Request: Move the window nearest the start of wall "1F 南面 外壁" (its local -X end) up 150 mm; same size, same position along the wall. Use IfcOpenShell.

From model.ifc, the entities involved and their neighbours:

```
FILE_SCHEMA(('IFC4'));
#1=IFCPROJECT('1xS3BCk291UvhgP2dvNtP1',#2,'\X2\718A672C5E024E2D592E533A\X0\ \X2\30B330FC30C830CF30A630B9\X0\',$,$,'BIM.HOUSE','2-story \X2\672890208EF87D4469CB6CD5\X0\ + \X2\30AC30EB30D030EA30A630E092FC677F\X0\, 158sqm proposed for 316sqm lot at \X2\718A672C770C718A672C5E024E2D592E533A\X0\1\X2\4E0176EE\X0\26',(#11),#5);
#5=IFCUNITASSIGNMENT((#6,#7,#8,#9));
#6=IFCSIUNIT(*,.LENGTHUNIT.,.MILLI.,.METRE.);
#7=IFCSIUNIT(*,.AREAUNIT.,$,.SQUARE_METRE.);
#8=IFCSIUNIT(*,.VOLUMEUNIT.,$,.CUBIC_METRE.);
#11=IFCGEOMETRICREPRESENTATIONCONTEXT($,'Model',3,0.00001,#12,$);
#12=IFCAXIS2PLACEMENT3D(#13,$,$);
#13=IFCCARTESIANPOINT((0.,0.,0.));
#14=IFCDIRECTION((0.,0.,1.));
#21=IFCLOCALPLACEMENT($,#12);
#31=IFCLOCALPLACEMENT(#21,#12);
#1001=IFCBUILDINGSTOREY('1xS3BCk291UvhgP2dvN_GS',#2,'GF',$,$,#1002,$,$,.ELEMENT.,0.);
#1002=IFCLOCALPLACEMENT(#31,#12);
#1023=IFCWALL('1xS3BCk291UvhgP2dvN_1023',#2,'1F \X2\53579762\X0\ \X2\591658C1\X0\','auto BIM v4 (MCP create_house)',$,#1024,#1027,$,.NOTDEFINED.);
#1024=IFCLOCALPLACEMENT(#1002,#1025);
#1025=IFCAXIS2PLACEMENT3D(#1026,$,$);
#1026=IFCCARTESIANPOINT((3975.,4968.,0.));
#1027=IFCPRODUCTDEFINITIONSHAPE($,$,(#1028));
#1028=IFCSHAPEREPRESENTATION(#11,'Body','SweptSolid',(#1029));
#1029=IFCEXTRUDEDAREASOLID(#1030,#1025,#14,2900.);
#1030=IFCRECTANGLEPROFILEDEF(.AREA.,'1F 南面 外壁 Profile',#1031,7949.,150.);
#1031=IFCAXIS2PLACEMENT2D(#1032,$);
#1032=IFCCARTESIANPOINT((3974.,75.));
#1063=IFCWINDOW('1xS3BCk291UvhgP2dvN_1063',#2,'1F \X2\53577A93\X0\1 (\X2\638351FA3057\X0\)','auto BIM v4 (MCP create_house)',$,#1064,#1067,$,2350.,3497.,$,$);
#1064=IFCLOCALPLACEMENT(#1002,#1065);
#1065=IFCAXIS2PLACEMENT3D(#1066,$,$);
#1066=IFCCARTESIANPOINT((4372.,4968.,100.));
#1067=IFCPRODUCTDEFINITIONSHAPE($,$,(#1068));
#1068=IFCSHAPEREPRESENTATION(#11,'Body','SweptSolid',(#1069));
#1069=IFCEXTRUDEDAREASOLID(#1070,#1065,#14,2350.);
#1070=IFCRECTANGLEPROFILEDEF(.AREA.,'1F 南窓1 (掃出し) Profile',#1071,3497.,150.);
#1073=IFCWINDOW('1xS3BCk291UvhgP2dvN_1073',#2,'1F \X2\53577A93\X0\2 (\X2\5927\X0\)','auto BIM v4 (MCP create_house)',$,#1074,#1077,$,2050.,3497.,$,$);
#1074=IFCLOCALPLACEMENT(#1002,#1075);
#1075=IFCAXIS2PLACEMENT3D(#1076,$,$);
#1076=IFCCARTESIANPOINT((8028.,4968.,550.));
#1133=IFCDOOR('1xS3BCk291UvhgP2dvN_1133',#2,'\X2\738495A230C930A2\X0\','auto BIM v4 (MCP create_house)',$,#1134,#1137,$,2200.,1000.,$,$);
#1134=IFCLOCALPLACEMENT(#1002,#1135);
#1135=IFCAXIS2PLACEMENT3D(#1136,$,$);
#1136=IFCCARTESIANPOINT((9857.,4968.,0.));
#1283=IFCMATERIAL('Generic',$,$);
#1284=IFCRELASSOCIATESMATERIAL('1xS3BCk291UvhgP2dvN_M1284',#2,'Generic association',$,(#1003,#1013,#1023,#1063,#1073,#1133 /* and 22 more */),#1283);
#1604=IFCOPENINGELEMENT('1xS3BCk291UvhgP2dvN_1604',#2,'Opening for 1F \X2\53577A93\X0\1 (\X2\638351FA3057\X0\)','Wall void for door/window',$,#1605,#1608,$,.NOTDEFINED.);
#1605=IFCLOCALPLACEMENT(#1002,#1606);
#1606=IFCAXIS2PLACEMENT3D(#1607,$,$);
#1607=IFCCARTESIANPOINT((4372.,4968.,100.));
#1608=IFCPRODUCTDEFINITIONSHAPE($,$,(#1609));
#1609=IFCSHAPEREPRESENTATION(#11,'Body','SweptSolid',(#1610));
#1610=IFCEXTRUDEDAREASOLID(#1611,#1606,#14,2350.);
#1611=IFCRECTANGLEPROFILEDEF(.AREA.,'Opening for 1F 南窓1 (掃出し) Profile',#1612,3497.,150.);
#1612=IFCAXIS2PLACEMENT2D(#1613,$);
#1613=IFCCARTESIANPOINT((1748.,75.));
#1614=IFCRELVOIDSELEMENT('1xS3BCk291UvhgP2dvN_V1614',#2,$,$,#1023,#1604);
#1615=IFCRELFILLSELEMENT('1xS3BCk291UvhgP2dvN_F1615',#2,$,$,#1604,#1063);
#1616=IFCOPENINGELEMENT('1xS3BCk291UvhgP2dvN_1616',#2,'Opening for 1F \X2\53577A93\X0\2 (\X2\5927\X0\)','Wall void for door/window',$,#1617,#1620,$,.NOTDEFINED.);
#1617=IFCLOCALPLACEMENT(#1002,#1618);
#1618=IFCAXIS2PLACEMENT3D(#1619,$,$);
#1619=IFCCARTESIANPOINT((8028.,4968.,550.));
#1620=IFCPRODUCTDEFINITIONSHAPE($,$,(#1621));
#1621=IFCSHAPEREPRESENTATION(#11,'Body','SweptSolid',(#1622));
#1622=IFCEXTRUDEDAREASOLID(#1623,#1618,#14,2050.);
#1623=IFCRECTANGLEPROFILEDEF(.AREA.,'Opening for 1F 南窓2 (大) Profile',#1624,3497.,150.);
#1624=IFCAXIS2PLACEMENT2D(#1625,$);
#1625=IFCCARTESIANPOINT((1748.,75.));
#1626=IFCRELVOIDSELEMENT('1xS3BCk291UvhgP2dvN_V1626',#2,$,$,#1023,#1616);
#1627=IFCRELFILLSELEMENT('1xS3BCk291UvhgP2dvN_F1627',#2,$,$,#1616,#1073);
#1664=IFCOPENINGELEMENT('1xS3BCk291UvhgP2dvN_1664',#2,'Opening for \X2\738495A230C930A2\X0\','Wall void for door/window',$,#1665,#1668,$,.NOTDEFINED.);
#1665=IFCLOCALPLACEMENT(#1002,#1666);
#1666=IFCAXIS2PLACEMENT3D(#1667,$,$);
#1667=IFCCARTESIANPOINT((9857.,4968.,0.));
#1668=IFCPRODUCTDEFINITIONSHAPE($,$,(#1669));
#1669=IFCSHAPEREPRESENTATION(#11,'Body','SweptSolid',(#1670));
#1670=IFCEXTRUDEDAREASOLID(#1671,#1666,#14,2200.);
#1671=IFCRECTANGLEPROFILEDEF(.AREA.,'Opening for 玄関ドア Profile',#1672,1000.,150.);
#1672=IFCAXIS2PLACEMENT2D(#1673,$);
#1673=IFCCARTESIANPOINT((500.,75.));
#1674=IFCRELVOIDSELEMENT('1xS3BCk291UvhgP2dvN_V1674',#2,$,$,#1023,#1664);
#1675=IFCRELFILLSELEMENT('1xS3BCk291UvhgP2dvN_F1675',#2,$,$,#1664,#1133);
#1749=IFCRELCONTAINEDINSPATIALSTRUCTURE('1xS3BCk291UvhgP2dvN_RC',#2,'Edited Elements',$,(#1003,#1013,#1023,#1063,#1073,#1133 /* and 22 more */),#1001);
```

```python
import numpy as np
import ifcopenshell
import ifcopenshell.api.geometry
import ifcopenshell.util.placement
import ifcopenshell.util.unit

model = ifcopenshell.open("model.ifc")
unit_scale = ifcopenshell.util.unit.calculate_unit_scale(model)

window = model.by_id(1063)
opening = window.FillsVoids[0].RelatingOpeningElement
dz = 0.15 / unit_scale

shift = np.array([0.0, 0.0, dz])
# The window is not placed relative to its opening, so move both.
for product in (opening, window):
    matrix = ifcopenshell.util.placement.get_local_placement(product.ObjectPlacement)
    matrix[:3, 3] += shift
    ifcopenshell.api.geometry.edit_object_placement(model, product=product, matrix=matrix, is_si=False)

print(f"moved by {dz * unit_scale:+.3f} m")

model.write("model_rev.ifc")
```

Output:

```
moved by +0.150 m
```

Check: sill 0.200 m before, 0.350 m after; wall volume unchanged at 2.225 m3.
